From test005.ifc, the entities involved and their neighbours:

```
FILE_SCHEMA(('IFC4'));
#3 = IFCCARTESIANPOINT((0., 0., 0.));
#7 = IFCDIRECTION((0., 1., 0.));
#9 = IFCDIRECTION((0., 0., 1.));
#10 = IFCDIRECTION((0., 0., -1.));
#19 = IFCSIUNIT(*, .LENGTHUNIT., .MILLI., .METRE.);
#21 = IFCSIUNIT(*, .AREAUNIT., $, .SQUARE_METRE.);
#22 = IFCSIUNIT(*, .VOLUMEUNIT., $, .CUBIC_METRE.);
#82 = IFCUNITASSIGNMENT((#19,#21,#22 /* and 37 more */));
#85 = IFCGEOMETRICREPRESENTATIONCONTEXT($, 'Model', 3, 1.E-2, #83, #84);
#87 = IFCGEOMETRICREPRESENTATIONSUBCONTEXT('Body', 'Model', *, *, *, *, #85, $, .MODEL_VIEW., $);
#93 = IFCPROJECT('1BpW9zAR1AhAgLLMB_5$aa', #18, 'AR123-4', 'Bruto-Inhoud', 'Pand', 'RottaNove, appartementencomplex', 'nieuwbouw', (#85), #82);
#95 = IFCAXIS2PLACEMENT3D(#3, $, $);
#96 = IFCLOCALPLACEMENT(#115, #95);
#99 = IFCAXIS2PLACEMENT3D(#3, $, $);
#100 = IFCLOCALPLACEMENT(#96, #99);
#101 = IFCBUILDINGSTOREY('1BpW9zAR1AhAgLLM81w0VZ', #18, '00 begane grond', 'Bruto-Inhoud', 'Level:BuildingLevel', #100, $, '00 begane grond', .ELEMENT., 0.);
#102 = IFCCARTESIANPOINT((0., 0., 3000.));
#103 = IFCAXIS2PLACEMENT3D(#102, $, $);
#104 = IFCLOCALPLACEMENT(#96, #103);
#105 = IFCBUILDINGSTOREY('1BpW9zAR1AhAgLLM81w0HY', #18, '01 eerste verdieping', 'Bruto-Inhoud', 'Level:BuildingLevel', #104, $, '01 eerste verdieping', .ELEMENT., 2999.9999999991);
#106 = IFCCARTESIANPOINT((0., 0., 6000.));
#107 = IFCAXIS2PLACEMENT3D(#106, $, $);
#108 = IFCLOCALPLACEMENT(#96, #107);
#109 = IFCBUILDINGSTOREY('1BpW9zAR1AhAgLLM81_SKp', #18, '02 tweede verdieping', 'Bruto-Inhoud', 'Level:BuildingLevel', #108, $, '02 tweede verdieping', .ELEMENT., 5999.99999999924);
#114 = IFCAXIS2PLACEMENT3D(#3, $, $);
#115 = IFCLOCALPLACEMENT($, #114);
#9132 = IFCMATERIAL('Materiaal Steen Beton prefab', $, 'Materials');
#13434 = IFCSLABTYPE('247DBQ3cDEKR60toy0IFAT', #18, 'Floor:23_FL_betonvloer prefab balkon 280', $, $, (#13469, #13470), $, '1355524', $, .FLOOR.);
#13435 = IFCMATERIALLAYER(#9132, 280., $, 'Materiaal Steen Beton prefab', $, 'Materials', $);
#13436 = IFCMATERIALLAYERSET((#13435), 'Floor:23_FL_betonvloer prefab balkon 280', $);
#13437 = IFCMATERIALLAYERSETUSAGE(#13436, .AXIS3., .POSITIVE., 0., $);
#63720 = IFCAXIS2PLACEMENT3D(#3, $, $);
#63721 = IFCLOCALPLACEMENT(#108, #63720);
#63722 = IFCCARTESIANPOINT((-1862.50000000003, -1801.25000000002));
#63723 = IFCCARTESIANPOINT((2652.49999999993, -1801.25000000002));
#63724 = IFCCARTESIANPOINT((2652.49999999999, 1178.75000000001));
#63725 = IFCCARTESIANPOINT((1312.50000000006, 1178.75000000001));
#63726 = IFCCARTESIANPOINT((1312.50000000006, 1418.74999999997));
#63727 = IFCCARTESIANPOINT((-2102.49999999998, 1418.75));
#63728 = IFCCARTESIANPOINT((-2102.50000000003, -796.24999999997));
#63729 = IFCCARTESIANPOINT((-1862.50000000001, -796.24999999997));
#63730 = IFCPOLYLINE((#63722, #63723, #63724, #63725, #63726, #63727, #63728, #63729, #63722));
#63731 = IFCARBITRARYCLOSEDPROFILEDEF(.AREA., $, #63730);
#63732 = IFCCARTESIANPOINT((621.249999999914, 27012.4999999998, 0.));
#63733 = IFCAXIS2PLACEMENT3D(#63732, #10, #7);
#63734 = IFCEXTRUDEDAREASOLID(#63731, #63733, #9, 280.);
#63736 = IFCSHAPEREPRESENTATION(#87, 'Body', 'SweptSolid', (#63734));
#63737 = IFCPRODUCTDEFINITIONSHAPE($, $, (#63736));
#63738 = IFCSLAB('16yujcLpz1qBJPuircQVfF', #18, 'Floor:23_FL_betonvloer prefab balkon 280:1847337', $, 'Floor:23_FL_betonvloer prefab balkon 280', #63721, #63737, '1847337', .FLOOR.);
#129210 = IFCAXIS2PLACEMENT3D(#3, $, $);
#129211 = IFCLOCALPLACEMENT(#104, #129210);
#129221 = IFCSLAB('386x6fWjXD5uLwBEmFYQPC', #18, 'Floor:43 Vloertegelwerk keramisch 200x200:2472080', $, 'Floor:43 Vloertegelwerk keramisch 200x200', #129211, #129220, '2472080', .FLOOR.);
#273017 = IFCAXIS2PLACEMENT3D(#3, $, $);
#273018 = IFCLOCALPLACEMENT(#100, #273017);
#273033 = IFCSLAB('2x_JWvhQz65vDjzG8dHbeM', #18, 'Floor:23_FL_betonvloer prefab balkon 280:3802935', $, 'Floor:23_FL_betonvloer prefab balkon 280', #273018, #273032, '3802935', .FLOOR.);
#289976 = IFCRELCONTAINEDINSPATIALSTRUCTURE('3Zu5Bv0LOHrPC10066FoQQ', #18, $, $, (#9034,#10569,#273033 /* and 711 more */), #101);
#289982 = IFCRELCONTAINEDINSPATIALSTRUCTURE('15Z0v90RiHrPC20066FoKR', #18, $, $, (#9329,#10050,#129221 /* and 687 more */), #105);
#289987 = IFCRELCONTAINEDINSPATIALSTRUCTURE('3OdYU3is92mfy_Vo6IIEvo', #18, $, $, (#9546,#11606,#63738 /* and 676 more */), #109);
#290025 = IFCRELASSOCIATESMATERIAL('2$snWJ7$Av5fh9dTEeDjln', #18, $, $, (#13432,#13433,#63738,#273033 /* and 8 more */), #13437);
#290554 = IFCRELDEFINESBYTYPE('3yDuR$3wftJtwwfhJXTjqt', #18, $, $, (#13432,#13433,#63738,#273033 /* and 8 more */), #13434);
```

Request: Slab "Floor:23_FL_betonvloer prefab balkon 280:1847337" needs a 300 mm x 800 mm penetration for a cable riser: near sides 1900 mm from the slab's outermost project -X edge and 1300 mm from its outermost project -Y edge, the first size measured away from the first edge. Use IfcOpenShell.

```python
import numpy as np
import ifcopenshell
import ifcopenshell.api.feature
import ifcopenshell.api.geometry
import ifcopenshell.api.root
import ifcopenshell.geom
import ifcopenshell.util.placement
import ifcopenshell.util.representation
import ifcopenshell.util.shape
import ifcopenshell.util.unit

model = ifcopenshell.open("test005.ifc")
unit_scale = ifcopenshell.util.unit.calculate_unit_scale(model)
settings = ifcopenshell.geom.settings()


def volume(element):
    """Net volume in cubic metres, openings subtracted."""
    shape = ifcopenshell.geom.create_shape(settings, element)
    return ifcopenshell.util.shape.get_volume(shape.geometry)


slab = model.by_guid("16yujcLpz1qBJPuircQVfF")
before = volume(slab)

# Extent in the slab's own axes, in metres. The edges named are its -X and -Y sides.
slab_shape = ifcopenshell.geom.create_shape(settings, slab)
vertices = ifcopenshell.util.shape.get_vertices(slab_shape.geometry)
x_min, y_min, bottom = vertices.min(axis=0)
top = vertices[:, 2].max()

opening = ifcopenshell.api.root.create_entity(model, ifc_class="IfcOpeningElement", name="Cable riser opening", predefined_type="OPENING")
context = ifcopenshell.util.representation.get_context(model, "Model", "Body", "MODEL_VIEW")
width, depth = 0.3, 0.8
outline = [(0.0, 0.0), (width, 0.0), (width, depth), (0.0, depth), (0.0, 0.0)]
# Overshoot both faces by 50 mm so the cut is clean.
shape = ifcopenshell.api.geometry.add_slab_representation(
    model, context=context, depth=top - bottom + 0.1, polyline=outline
)
ifcopenshell.api.geometry.assign_representation(model, product=opening, representation=shape)

matrix = ifcopenshell.util.placement.get_local_placement(slab.ObjectPlacement)
matrix[:, 3] = matrix @ np.append(np.array([x_min + 1.9, y_min + 1.3, bottom - 0.05]) / unit_scale, 1.0)
ifcopenshell.api.geometry.edit_object_placement(model, product=opening, matrix=matrix, is_si=False)
ifcopenshell.api.feature.add_feature(model, feature=opening, element=slab)

after = volume(slab)

print(f"slab volume {before:.3f} -> {after:.3f} m3")

model.write("test005_updated.ifc")
```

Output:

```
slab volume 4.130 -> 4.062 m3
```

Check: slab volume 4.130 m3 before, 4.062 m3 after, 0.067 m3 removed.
